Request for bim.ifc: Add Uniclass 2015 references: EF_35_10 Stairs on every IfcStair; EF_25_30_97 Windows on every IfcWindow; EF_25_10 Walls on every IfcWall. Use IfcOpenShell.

First a look at what the model holds.

```python
import ifcopenshell

model = ifcopenshell.open("bim.ifc")
print(model.schema)
print("classifications:", [c.Name for c in model.by_type("IfcClassification")])
for ifc_class in ("IfcDoor", "IfcRoof", "IfcStair", "IfcWall", "IfcWindow"):
    print(ifc_class, len(model.by_type(ifc_class)))
```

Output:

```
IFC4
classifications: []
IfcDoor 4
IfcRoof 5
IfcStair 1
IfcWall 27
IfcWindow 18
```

```python
import ifcopenshell
import ifcopenshell.api.classification

model = ifcopenshell.open("bim.ifc")

system = ifcopenshell.api.classification.add_classification(model, classification="Uniclass 2015")

codes = {
    "IfcStair": ("EF_35_10", "Stairs"),
    "IfcWindow": ("EF_25_30_97", "Windows"),
    "IfcWall": ("EF_25_10", "Walls"),
}
for ifc_class, (code, name) in codes.items():
    products = model.by_type(ifc_class)
    ifcopenshell.api.classification.add_reference(
        model, products=products, classification=system, identification=code, name=name
    )
    print(code, len(products))

model.write("bim-out.ifc")
```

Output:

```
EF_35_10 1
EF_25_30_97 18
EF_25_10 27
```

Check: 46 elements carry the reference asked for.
